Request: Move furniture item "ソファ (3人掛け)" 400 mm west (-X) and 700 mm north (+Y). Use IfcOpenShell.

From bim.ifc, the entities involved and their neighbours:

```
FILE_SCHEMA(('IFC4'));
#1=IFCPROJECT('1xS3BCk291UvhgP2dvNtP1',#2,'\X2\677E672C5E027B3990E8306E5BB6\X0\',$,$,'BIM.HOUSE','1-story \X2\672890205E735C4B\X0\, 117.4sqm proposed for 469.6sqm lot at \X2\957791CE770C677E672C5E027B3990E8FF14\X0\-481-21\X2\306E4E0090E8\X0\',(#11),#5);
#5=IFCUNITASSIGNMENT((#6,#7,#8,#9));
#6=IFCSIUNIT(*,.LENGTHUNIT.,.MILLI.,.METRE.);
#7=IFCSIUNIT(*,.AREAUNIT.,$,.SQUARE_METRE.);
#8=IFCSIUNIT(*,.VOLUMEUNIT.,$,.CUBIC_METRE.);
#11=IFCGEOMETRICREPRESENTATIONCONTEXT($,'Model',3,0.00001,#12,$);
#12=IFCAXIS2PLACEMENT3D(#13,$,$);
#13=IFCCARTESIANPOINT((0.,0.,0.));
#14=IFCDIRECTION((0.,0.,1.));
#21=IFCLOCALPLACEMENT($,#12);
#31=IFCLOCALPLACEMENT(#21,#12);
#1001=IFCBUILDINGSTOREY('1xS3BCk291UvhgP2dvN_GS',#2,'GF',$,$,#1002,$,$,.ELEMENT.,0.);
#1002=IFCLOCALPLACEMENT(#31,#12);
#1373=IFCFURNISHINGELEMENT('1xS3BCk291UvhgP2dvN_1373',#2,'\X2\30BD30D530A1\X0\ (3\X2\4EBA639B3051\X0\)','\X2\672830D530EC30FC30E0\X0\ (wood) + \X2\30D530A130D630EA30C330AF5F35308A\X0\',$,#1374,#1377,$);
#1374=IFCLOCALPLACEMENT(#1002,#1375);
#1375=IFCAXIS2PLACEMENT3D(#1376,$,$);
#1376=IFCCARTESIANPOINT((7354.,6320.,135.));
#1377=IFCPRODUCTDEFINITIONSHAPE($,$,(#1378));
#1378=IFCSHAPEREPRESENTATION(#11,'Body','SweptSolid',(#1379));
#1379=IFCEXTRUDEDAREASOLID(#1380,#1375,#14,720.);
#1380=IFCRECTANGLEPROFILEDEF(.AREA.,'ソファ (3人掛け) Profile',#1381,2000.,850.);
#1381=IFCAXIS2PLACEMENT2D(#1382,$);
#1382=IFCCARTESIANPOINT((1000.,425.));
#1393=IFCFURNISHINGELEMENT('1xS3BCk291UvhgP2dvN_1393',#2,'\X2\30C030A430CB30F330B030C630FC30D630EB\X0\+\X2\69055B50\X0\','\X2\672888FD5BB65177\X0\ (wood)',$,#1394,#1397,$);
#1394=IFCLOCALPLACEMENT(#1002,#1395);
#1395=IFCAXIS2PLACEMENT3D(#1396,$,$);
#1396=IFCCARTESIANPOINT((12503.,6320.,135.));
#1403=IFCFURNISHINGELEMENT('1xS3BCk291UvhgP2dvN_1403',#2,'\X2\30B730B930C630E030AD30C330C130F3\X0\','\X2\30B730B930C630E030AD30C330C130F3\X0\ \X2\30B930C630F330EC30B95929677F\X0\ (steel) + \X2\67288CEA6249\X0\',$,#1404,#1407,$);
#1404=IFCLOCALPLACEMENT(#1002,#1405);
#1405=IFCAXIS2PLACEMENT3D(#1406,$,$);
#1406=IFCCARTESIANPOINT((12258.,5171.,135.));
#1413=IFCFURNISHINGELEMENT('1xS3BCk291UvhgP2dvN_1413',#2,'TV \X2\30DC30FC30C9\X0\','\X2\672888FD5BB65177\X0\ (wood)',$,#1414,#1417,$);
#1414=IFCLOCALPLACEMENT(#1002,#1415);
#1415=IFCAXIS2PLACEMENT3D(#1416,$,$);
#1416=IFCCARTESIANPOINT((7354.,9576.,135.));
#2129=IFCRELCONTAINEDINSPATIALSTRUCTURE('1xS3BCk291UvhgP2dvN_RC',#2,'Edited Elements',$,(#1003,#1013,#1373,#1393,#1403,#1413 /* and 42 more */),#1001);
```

```python
import ifcopenshell
import ifcopenshell.api.geometry
import ifcopenshell.util.placement

model = ifcopenshell.open("bim.ifc")

item = model.by_guid("1xS3BCk291UvhgP2dvN_1373")
matrix = ifcopenshell.util.placement.get_local_placement(item.ObjectPlacement)
matrix[0, 3] -= 400.0
matrix[1, 3] += 700.0
ifcopenshell.api.geometry.edit_object_placement(model, product=item, matrix=matrix, is_si=False)

print(ifcopenshell.util.placement.get_local_placement(item.ObjectPlacement).round(3) + 0.0)

model.write("bim_edited.ifc")
```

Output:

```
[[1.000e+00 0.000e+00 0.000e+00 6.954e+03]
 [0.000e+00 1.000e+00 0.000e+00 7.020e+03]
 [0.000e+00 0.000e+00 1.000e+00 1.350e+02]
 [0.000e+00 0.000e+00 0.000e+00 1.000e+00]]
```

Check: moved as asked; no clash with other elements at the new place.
